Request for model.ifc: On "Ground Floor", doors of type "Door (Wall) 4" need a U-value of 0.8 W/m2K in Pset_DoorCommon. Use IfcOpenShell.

First a look at what the model holds.

```python
import ifcopenshell
import ifcopenshell.util.element

model = ifcopenshell.open("model.ifc")
print(model.schema)
storey = next(s for s in model.by_type("IfcBuildingStorey") if s.Name == "Ground Floor")
doors = [e for e in ifcopenshell.util.element.get_decomposition(storey) if e.is_a("IfcDoor")]
seen = {}
for e in doors:
    element_type = ifcopenshell.util.element.get_type(e)
    key = (element_type.Name if element_type != e and element_type else None, ifcopenshell.util.element.get_pset(e, "Pset_DoorCommon", "ThermalTransmittance"))
    seen[key] = seen.get(key, 0) + 1
for (name, value), count in sorted(seen.items(), key=str):
    print(count, "x", name, "|", value)
```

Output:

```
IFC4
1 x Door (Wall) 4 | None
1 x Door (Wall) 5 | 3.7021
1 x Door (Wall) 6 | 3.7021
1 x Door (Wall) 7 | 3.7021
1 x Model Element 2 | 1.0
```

```python
import ifcopenshell
import ifcopenshell.api.pset
import ifcopenshell.util.element

model = ifcopenshell.open("model.ifc")

storey = next(s for s in model.by_type("IfcBuildingStorey") if s.Name == "Ground Floor")
doors = [e for e in ifcopenshell.util.element.get_decomposition(storey) if e.is_a("IfcDoor")]

count = 0
for e in doors:
    element_type = ifcopenshell.util.element.get_type(e)
    if element_type in (None, e) or element_type.Name != "Door (Wall) 4":
        continue
    # add_pset returns the element's existing set when there is one.
    pset = ifcopenshell.api.pset.add_pset(model, product=e, name="Pset_DoorCommon")
    ifcopenshell.api.pset.edit_pset(model, pset=pset, properties={"ThermalTransmittance": 0.8})
    count += 1

print(count, "doors updated")

model.write("model_edited.ifc")
```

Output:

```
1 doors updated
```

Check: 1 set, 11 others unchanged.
